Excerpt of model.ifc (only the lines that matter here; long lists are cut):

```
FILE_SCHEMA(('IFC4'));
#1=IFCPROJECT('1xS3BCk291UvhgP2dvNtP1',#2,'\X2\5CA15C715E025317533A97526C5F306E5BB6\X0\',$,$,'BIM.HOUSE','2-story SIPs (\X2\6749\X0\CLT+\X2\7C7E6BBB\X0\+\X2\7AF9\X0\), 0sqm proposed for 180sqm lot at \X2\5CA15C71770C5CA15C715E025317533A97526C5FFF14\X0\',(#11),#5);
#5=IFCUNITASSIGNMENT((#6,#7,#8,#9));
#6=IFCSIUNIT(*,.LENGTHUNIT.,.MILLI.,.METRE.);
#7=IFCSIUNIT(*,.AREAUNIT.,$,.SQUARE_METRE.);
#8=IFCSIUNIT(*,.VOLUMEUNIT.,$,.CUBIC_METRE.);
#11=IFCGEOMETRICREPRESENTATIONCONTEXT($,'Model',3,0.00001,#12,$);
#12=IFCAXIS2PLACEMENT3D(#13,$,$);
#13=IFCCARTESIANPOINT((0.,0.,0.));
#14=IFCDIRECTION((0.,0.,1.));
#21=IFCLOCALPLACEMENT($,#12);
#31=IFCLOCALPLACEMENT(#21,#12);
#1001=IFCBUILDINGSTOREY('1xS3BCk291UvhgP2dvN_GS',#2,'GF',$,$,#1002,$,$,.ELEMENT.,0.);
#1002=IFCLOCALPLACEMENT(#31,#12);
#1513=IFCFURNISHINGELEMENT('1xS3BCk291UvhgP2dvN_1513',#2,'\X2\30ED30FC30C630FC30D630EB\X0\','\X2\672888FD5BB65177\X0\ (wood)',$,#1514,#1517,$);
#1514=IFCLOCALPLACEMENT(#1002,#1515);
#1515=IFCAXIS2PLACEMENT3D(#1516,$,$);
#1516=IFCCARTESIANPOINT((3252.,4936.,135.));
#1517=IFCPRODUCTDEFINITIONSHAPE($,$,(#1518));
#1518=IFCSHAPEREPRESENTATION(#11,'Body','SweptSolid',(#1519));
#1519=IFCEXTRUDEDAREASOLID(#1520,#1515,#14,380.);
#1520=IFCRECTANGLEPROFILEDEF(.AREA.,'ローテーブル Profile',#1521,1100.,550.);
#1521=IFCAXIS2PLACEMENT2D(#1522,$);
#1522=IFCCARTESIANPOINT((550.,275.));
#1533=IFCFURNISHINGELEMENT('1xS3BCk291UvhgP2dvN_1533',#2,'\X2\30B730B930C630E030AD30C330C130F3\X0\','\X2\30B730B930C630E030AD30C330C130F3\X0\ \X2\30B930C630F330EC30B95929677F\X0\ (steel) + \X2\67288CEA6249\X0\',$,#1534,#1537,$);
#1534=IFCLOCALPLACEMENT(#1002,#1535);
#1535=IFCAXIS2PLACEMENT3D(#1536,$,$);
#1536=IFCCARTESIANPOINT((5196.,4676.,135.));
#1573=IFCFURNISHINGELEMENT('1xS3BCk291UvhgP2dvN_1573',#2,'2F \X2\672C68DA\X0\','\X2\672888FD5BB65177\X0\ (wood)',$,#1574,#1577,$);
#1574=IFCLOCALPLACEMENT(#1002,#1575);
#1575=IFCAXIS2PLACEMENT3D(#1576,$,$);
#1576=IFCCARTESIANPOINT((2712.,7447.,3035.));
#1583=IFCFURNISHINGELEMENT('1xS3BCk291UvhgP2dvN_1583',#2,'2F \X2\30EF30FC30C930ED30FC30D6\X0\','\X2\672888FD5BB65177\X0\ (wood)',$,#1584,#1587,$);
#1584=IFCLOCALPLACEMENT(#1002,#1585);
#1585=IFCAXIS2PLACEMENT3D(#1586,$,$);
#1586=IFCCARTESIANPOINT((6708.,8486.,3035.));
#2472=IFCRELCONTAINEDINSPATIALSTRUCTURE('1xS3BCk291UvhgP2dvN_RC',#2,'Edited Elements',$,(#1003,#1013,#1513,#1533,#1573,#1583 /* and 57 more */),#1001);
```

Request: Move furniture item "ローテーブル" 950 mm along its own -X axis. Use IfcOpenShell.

```python
import ifcopenshell
import ifcopenshell.api.geometry
import ifcopenshell.util.placement
import ifcopenshell.util.unit

model = ifcopenshell.open("model.ifc")
unit_scale = ifcopenshell.util.unit.calculate_unit_scale(model)

item = model.by_id(1513)
matrix = ifcopenshell.util.placement.get_local_placement(item.ObjectPlacement)
matrix[:3, 3] -= matrix[:3, 0] * 0.95 / unit_scale
ifcopenshell.api.geometry.edit_object_placement(model, product=item, matrix=matrix, is_si=False)

print(ifcopenshell.util.placement.get_local_placement(item.ObjectPlacement).round(3) + 0.0)

model.write("model_rev.ifc")
```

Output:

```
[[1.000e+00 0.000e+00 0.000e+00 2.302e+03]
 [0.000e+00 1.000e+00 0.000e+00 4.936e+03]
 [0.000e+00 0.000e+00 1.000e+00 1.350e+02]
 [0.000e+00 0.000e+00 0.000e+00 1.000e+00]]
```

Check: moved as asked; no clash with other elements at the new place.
